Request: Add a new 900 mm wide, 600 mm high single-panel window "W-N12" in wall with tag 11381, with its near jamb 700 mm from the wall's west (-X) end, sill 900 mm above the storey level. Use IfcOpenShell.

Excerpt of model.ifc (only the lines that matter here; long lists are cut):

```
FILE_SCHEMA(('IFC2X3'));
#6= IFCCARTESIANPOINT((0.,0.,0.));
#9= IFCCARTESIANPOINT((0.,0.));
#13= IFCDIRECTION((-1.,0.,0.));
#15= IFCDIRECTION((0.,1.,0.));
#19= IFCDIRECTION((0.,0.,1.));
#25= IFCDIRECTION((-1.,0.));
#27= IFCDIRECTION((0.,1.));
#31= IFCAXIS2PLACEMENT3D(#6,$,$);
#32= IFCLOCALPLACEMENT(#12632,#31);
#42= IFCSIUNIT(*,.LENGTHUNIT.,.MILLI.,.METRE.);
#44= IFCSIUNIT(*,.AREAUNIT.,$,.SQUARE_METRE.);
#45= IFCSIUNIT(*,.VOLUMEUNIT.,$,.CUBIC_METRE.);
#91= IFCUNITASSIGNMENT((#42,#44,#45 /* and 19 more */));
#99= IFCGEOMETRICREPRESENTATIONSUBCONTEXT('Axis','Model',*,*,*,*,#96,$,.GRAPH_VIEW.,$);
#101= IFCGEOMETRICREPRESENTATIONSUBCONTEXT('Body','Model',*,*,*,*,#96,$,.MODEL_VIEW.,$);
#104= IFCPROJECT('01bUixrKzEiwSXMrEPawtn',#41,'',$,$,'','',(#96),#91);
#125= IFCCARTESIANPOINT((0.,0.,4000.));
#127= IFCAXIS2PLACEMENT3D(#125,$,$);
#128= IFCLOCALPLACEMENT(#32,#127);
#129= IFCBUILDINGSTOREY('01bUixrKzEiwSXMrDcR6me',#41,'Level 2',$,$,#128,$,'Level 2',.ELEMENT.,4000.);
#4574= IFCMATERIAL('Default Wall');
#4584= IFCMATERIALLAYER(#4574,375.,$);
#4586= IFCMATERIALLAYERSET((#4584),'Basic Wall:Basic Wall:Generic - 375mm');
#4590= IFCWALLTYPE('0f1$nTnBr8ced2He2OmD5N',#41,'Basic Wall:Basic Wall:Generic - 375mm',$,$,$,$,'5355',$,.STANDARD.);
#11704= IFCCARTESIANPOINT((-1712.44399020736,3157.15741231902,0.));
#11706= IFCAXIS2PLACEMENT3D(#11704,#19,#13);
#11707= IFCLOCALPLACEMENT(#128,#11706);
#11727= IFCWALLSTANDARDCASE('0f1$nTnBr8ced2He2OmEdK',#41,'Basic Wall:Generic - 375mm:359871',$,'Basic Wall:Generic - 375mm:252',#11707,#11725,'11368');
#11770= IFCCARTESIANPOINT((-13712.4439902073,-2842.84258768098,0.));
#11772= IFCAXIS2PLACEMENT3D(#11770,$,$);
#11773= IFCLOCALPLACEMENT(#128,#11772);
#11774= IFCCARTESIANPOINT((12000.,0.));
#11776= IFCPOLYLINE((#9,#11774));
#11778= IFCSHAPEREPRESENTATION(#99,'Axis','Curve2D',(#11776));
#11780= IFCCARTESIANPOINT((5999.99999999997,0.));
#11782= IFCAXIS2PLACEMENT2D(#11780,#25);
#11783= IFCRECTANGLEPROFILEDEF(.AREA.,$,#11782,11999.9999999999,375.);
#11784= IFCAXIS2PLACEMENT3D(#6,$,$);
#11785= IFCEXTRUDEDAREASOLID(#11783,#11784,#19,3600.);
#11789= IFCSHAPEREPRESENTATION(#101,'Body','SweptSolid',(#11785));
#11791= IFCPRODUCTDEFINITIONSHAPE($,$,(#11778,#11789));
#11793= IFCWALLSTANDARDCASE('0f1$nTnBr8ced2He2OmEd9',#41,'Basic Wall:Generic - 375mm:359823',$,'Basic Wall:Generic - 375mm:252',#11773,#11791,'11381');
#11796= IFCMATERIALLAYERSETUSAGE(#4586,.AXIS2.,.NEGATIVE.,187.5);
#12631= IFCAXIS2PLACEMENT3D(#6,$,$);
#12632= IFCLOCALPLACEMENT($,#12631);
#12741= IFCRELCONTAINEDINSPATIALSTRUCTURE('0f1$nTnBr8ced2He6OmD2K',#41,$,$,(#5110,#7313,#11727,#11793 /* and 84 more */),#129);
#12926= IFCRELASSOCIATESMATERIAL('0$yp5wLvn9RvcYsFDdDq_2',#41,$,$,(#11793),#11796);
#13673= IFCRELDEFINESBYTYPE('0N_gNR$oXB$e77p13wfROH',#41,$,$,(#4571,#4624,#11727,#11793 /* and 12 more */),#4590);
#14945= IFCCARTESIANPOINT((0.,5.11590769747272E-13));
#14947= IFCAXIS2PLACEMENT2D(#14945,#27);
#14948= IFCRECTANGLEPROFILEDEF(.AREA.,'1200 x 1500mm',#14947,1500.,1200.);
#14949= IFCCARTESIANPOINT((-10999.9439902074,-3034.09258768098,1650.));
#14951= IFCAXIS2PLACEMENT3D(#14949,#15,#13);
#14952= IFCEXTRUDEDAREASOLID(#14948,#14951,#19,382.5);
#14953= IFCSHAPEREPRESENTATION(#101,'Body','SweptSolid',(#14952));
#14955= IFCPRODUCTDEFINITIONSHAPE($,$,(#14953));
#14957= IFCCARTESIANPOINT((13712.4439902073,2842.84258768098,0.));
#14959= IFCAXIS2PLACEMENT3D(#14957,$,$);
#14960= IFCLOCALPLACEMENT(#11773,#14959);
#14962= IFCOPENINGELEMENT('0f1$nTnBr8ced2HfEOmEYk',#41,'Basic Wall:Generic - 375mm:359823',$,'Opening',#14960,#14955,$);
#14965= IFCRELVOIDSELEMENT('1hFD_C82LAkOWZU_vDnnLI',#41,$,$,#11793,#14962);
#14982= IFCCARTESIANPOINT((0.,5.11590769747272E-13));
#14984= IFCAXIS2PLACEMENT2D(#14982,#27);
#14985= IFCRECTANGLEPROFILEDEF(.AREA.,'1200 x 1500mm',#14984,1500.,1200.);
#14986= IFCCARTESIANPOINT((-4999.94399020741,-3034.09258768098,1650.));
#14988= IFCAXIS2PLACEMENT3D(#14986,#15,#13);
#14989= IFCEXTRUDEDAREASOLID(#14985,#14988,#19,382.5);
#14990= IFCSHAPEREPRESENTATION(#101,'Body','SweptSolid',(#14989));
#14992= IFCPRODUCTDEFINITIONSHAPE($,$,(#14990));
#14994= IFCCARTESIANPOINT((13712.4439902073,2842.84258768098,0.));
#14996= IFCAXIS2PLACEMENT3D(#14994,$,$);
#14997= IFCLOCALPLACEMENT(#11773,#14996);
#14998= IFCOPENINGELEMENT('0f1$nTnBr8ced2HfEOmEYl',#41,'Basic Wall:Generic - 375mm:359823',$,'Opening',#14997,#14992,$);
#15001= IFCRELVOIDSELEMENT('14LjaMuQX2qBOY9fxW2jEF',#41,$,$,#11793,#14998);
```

```python
import numpy as np
import ifcopenshell
import ifcopenshell.api.feature
import ifcopenshell.api.geometry
import ifcopenshell.api.root
import ifcopenshell.api.spatial
import ifcopenshell.api.type
import ifcopenshell.geom
import ifcopenshell.util.element
import ifcopenshell.util.placement
import ifcopenshell.util.representation
import ifcopenshell.util.shape
import ifcopenshell.util.unit

model = ifcopenshell.open("model.ifc")
unit_scale = ifcopenshell.util.unit.calculate_unit_scale(model)
settings = ifcopenshell.geom.settings()


def volume(element):
    """Net volume in cubic metres, openings subtracted."""
    shape = ifcopenshell.geom.create_shape(settings, element)
    return ifcopenshell.util.shape.get_volume(shape.geometry)


wall = model.by_guid("0f1$nTnBr8ced2He2OmEd9")
storey = ifcopenshell.util.element.get_container(wall, ifc_class="IfcBuildingStorey")
context = ifcopenshell.util.representation.get_context(model, "Model", "Body", "MODEL_VIEW")
before = volume(wall)

width, height, from_end, sill = 0.9, 0.6, 0.7, 0.9  # metres

# The wall runs along its own X axis, and the end named is its -X end.
wall_shape = ifcopenshell.geom.create_shape(settings, wall)
x, y, z = ifcopenshell.util.shape.get_vertices(wall_shape.geometry).T
start = x.min() + from_end
face, thickness = float(y.min()), float(y.max() - y.min())
wall_matrix = ifcopenshell.util.placement.get_local_placement(wall.ObjectPlacement)
level = ifcopenshell.util.placement.get_local_placement(storey.ObjectPlacement)[2, 3]


def in_wall(x, y):
    """Placement at x, y metres in the wall's axes, at sill height."""
    matrix = wall_matrix.copy()
    matrix[:, 3] = wall_matrix @ np.array([x / unit_scale, y / unit_scale, 0.0, 1.0])
    matrix[2, 3] = level + sill / unit_scale
    return matrix


# Opening: a box that overshoots both wall faces by 50 mm.
opening = ifcopenshell.api.root.create_entity(model, ifc_class="IfcOpeningElement")
box = ifcopenshell.api.geometry.add_wall_representation(
    model, context=context, length=width, height=height, thickness=thickness + 0.1
)
ifcopenshell.api.geometry.assign_representation(model, product=opening, representation=box)
ifcopenshell.api.geometry.edit_object_placement(model, product=opening, matrix=in_wall(start, face - 0.05), is_si=False)
ifcopenshell.api.feature.add_feature(model, feature=opening, element=wall)

window = ifcopenshell.api.root.create_entity(model, ifc_class="IfcWindow", name="W-N12")
window.OverallWidth, window.OverallHeight = width / unit_scale, height / unit_scale
body = ifcopenshell.api.geometry.add_window_representation(
    model,
    context=context,
    overall_width=window.OverallWidth,
    overall_height=window.OverallHeight,
    partition_type="SINGLE_PANEL",
)
ifcopenshell.api.geometry.assign_representation(model, product=window, representation=body)
ifcopenshell.api.spatial.assign_container(model, products=[window], relating_structure=storey)
fills = ifcopenshell.api.feature.add_filling(model, opening=opening, element=window)
fills.OwnerHistory = window.OwnerHistory  # required in IFC2X3

# IFC2X3 keeps the operation on the window style.
style = ifcopenshell.api.root.create_entity(model, ifc_class="IfcWindowStyle", name="W-N12")
style.OperationType, style.ConstructionType = "SINGLE_PANEL", "NOTDEFINED"
style.ParameterTakesPrecedence = style.Sizeable = False
ifcopenshell.api.type.assign_type(model, related_objects=[window], relating_type=style)

# Centre the window in the wall's thickness.
ifcopenshell.api.geometry.edit_object_placement(model, product=window, matrix=in_wall(start, face), is_si=False)
window_shape = ifcopenshell.geom.create_shape(settings, window)
depth = ifcopenshell.util.shape.get_vertices(window_shape.geometry)[:, 1]
offset = face + thickness / 2 - (depth.min() + depth.max()) / 2
ifcopenshell.api.geometry.edit_object_placement(model, product=window, matrix=in_wall(start, offset), is_si=False)

after = volume(wall)

print(f"wall volume {before:.3f} -> {after:.3f} m3")

model.write("model-out.ifc")
```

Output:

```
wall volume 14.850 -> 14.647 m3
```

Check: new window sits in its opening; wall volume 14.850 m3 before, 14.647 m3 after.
